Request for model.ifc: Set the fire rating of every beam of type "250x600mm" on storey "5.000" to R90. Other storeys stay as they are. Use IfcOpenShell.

First a look at what the model holds.

```python
import ifcopenshell
import ifcopenshell.util.element

model = ifcopenshell.open("model.ifc")
print(model.schema)
storey = next(s for s in model.by_type("IfcBuildingStorey") if s.Name == "5.000")
beams = [e for e in ifcopenshell.util.element.get_decomposition(storey) if e.is_a("IfcBeam")]
seen = {}
for e in beams:
    element_type = ifcopenshell.util.element.get_type(e)
    key = (element_type.Name if element_type != e and element_type else None, ifcopenshell.util.element.get_pset(e, "Pset_BeamCommon", "FireRating"))
    seen[key] = seen.get(key, 0) + 1
for (name, value), count in sorted(seen.items(), key=str):
    print(count, "x", name, "|", value)
```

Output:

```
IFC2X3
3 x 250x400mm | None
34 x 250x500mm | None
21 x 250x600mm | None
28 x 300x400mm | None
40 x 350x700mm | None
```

```python
import ifcopenshell
import ifcopenshell.api.pset
import ifcopenshell.util.element

model = ifcopenshell.open("model.ifc")

storey = next(s for s in model.by_type("IfcBuildingStorey") if s.Name == "5.000")
beams = [e for e in ifcopenshell.util.element.get_decomposition(storey) if e.is_a("IfcBeam")]

count = 0
for e in beams:
    element_type = ifcopenshell.util.element.get_type(e)
    if element_type in (None, e) or element_type.Name != "250x600mm":
        continue
    # add_pset returns the element's existing set when there is one.
    pset = ifcopenshell.api.pset.add_pset(model, product=e, name="Pset_BeamCommon")
    ifcopenshell.api.pset.edit_pset(model, pset=pset, properties={"FireRating": "R90"})
    count += 1

print(count, "beams updated")

model.write("model_edited.ifc")
```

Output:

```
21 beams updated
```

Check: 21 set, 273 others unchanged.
